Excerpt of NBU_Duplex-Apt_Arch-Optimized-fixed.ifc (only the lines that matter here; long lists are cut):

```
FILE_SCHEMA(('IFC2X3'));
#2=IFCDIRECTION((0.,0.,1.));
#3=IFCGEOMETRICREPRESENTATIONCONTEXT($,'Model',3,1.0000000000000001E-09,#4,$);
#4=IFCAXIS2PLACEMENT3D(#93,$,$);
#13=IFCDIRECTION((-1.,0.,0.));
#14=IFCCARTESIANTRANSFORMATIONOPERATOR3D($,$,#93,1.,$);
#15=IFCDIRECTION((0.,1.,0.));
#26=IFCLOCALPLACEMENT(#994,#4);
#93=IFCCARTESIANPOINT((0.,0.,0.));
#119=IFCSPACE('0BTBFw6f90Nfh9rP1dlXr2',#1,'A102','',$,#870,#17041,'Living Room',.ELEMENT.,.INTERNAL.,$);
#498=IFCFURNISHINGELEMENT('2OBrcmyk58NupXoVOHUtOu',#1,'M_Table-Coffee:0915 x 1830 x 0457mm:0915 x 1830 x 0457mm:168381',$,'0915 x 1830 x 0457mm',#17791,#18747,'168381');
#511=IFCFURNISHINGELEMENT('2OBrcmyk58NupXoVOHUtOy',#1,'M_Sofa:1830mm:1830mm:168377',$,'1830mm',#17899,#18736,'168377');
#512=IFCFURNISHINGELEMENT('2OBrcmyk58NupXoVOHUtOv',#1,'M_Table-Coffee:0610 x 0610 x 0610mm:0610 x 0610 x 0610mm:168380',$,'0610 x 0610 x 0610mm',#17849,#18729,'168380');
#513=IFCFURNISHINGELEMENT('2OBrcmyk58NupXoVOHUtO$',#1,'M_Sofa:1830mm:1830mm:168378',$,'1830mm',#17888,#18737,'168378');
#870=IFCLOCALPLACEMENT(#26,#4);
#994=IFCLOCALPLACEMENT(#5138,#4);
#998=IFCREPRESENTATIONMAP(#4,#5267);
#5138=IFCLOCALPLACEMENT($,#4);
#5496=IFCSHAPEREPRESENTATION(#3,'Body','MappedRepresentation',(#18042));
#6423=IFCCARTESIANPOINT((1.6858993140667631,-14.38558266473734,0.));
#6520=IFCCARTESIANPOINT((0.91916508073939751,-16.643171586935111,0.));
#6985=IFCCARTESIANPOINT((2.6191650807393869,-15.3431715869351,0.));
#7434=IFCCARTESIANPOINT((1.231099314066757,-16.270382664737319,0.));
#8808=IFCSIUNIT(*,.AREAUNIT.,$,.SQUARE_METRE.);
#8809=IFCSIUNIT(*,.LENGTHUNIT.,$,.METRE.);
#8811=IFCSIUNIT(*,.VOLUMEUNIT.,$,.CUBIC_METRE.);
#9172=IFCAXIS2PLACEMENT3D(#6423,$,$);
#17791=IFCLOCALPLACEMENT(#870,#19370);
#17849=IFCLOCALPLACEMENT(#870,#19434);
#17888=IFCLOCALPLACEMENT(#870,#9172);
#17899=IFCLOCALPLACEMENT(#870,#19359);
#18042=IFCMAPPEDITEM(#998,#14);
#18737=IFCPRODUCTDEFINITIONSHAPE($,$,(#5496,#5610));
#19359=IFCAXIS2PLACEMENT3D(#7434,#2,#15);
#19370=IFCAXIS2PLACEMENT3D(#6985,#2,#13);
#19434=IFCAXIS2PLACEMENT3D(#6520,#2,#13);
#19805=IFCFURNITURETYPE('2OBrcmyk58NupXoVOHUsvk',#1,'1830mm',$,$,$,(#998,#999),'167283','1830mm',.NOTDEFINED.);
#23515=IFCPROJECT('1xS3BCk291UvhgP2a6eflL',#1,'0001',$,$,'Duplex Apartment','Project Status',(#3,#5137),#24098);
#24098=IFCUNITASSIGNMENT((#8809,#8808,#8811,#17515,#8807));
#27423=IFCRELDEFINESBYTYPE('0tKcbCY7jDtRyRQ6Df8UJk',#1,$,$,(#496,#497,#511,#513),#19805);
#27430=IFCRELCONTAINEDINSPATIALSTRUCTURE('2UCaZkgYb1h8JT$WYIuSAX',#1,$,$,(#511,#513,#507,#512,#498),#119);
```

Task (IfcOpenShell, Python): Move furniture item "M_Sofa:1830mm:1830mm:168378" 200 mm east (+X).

```python
import ifcopenshell
import ifcopenshell.api.geometry
import ifcopenshell.util.placement

model = ifcopenshell.open("NBU_Duplex-Apt_Arch-Optimized-fixed.ifc")

item = model.by_guid("2OBrcmyk58NupXoVOHUtO$")
matrix = ifcopenshell.util.placement.get_local_placement(item.ObjectPlacement)
matrix[0, 3] += 0.2
ifcopenshell.api.geometry.edit_object_placement(model, product=item, matrix=matrix, is_si=False)

print(ifcopenshell.util.placement.get_local_placement(item.ObjectPlacement).round(3) + 0.0)

model.write("NBU_Duplex-Apt_Arch-Optimized-fixed-out.ifc")
```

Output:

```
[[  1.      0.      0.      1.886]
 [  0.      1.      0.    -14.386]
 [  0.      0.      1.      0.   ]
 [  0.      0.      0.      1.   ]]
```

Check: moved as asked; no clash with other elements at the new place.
